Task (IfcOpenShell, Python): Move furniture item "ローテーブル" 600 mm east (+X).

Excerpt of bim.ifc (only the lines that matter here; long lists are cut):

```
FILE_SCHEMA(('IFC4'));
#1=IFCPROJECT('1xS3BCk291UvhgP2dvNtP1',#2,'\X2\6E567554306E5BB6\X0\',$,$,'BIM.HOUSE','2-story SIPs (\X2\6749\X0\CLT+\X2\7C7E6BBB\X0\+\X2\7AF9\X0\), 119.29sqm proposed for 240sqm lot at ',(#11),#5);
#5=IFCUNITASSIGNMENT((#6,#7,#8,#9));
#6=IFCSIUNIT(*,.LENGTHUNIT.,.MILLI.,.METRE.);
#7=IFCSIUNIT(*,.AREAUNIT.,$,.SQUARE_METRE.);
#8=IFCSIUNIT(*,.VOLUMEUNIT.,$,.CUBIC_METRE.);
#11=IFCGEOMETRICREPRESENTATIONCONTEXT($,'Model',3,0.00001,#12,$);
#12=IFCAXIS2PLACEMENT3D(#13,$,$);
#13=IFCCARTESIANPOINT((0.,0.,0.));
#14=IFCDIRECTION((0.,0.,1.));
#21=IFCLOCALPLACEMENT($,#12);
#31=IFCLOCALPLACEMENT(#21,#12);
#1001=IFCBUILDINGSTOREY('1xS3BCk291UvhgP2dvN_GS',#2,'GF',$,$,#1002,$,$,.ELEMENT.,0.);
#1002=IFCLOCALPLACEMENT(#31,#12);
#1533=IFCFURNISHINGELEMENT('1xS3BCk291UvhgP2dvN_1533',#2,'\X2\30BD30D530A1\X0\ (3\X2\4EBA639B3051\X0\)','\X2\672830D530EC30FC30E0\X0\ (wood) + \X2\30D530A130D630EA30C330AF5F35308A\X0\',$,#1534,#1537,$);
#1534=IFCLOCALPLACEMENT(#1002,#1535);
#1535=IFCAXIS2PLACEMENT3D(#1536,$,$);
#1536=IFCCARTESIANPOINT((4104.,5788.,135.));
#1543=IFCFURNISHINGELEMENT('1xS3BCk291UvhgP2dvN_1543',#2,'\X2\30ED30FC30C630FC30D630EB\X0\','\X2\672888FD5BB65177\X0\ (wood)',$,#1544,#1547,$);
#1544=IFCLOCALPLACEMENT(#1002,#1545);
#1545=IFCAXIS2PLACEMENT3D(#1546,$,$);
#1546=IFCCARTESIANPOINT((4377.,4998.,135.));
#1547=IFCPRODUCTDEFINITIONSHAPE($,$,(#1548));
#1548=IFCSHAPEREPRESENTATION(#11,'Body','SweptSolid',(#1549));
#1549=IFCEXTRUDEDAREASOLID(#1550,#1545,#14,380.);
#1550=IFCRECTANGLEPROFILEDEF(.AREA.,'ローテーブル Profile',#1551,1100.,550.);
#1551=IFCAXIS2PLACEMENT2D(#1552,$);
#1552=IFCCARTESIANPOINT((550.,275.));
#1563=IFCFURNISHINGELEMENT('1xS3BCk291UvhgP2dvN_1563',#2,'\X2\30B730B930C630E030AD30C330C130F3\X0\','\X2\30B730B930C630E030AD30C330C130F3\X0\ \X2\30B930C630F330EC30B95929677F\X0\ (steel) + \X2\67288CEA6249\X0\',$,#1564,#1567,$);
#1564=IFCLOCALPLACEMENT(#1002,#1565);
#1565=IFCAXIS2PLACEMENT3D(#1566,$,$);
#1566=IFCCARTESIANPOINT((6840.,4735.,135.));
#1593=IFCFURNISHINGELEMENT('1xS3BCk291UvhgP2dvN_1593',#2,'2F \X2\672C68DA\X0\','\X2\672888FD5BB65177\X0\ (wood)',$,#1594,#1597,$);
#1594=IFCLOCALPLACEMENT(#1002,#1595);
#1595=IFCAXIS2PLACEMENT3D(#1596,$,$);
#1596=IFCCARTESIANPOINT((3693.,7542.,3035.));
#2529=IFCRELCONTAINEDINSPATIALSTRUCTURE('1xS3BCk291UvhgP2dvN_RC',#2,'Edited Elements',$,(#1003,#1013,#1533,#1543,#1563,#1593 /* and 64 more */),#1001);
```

```python
import ifcopenshell
import ifcopenshell.api.geometry
import ifcopenshell.util.placement
import ifcopenshell.util.unit

model = ifcopenshell.open("bim.ifc")
unit_scale = ifcopenshell.util.unit.calculate_unit_scale(model)

item = model.by_guid("1xS3BCk291UvhgP2dvN_1543")
matrix = ifcopenshell.util.placement.get_local_placement(item.ObjectPlacement)
matrix[0, 3] += 0.6 / unit_scale
ifcopenshell.api.geometry.edit_object_placement(model, product=item, matrix=matrix, is_si=False)

print(ifcopenshell.util.placement.get_local_placement(item.ObjectPlacement).round(3) + 0.0)

model.write("bim_edited.ifc")
```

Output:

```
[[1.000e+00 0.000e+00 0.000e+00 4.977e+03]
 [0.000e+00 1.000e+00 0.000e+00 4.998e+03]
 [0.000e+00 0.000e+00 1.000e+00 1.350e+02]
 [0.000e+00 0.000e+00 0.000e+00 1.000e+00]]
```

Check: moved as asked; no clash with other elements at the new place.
